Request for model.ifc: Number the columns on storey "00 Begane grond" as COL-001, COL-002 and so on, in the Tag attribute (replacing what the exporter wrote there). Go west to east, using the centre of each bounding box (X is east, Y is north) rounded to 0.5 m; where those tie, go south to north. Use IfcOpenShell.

First a look at what the model holds.

```python
import ifcopenshell
import ifcopenshell.util.element
import ifcopenshell.util.placement

model = ifcopenshell.open("model.ifc")
print(model.schema)
storey = next(s for s in model.by_type("IfcBuildingStorey") if s.Name == "00 Begane grond")
columns = [e for e in ifcopenshell.util.element.get_decomposition(storey) if e.is_a("IfcColumn")]
for e in sorted(columns, key=lambda e: e.id()):
    origin = ifcopenshell.util.placement.get_local_placement(e.ObjectPlacement)[:3, 3]
    print(e.id(), e.Tag, e.Name, origin.round(2) + 0.0, sep=" | ")
```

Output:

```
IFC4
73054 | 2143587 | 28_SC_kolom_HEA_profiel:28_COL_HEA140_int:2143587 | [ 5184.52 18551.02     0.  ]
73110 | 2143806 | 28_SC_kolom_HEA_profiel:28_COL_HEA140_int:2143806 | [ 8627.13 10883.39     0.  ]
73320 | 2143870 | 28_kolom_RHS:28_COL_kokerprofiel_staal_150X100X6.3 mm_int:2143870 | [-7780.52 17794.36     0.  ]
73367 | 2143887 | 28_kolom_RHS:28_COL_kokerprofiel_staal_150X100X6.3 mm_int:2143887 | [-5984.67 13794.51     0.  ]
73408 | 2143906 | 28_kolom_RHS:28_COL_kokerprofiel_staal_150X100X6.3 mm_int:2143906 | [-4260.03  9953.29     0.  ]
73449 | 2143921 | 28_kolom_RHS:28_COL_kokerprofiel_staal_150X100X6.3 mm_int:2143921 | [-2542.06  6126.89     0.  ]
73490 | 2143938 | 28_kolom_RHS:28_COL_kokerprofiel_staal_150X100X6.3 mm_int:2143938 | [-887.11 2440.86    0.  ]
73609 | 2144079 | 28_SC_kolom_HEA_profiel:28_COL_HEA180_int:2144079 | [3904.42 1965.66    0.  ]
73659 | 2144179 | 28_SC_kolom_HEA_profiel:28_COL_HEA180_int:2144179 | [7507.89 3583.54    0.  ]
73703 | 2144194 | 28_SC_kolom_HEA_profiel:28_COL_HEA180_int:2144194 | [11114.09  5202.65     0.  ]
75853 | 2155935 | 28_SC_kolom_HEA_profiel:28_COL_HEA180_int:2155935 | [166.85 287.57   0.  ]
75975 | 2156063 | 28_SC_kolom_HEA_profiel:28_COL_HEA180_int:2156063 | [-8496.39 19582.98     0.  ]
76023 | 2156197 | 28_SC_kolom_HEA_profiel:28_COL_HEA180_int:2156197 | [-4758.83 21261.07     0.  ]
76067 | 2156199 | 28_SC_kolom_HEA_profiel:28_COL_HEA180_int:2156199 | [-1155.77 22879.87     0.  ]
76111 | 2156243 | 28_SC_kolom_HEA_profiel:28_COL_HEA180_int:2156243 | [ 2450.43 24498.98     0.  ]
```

```python
import ifcopenshell
import ifcopenshell.geom
import ifcopenshell.util.element
import ifcopenshell.util.shape

model = ifcopenshell.open("model.ifc")
settings = ifcopenshell.geom.settings()
settings.set("use-world-coords", True)


def centre(element):
    shape = ifcopenshell.geom.create_shape(settings, element)
    return ifcopenshell.util.shape.get_bbox_centroid(shape.geometry)


storey = next(s for s in model.by_type("IfcBuildingStorey") if s.Name == "00 Begane grond")
columns = [e for e in ifcopenshell.util.element.get_decomposition(storey) if e.is_a("IfcColumn")]

# Insertion points can sit at a corner or the storey origin, so sort by the geometry (in metres).
centres = {e: centre(e) for e in columns}
columns.sort(key=lambda e: (round(centres[e][0] / 0.5), centres[e][1]))

for i, e in enumerate(columns, start=1):
    number = f"COL-0{i:02d}"
    e.Tag = number
    print(e.id(), number)

model.write("model_v2.ifc")
```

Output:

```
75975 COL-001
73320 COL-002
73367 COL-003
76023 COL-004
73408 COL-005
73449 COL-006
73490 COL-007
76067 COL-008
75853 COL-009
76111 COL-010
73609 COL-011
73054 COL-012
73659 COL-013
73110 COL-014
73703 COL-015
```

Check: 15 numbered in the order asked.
